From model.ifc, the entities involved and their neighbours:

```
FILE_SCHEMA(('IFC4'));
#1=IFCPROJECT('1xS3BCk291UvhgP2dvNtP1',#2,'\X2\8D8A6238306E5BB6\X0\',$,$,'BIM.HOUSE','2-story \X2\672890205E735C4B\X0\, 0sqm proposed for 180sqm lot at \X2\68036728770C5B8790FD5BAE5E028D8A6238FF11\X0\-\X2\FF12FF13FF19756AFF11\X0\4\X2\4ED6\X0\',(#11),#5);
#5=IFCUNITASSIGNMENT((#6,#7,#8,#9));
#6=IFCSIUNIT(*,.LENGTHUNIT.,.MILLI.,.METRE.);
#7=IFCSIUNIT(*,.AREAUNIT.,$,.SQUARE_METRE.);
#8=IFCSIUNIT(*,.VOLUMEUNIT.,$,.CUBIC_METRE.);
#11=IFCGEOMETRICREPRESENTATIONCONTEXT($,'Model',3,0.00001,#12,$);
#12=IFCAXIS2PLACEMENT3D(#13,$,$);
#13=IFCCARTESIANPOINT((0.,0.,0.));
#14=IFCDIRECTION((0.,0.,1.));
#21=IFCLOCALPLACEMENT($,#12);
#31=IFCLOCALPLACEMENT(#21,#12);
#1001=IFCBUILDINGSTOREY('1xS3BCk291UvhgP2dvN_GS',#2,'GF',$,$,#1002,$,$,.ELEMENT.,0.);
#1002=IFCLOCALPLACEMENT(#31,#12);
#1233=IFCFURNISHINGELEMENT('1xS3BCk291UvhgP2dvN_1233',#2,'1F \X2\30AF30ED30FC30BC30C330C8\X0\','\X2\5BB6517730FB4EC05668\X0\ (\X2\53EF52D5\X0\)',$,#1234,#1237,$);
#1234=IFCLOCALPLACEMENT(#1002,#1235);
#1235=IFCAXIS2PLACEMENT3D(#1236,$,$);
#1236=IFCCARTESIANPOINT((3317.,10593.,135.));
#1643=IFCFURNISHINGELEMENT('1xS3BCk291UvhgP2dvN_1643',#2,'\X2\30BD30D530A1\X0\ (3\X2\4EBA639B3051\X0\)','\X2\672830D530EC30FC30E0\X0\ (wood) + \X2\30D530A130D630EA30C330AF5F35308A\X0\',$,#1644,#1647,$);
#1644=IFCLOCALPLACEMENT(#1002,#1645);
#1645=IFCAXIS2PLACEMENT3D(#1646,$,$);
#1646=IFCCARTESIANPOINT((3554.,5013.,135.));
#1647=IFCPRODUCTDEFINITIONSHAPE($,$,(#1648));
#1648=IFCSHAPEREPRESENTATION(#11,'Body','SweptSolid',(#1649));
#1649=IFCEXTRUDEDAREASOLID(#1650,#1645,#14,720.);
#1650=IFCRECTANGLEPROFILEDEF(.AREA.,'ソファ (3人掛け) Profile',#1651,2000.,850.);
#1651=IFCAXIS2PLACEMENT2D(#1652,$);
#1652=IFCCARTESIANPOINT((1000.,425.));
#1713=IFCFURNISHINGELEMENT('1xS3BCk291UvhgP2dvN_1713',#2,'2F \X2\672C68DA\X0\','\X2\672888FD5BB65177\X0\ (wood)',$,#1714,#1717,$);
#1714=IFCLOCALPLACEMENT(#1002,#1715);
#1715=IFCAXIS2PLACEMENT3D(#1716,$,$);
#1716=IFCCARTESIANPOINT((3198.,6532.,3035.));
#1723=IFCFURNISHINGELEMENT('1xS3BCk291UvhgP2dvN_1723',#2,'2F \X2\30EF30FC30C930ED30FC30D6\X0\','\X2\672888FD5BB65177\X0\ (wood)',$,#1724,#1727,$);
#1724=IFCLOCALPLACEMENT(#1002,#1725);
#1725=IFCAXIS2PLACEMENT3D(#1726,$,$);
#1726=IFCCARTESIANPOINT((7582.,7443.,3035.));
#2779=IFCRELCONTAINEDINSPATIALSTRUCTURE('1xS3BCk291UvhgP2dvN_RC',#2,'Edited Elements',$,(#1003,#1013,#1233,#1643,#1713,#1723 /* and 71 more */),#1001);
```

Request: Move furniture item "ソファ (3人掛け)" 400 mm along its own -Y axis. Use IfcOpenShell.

```python
import ifcopenshell
import ifcopenshell.api.geometry
import ifcopenshell.util.placement
import ifcopenshell.util.unit

model = ifcopenshell.open("model.ifc")
unit_scale = ifcopenshell.util.unit.calculate_unit_scale(model)

item = model.by_guid("1xS3BCk291UvhgP2dvN_1643")
matrix = ifcopenshell.util.placement.get_local_placement(item.ObjectPlacement)
matrix[:3, 3] -= matrix[:3, 1] * 0.4 / unit_scale
ifcopenshell.api.geometry.edit_object_placement(model, product=item, matrix=matrix, is_si=False)

print(ifcopenshell.util.placement.get_local_placement(item.ObjectPlacement).round(3) + 0.0)

model.write("model_updated.ifc")
```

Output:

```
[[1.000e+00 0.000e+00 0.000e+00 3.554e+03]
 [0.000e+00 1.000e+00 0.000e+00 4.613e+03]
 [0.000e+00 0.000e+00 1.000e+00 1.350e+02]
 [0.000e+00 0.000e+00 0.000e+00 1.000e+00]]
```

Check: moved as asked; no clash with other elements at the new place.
